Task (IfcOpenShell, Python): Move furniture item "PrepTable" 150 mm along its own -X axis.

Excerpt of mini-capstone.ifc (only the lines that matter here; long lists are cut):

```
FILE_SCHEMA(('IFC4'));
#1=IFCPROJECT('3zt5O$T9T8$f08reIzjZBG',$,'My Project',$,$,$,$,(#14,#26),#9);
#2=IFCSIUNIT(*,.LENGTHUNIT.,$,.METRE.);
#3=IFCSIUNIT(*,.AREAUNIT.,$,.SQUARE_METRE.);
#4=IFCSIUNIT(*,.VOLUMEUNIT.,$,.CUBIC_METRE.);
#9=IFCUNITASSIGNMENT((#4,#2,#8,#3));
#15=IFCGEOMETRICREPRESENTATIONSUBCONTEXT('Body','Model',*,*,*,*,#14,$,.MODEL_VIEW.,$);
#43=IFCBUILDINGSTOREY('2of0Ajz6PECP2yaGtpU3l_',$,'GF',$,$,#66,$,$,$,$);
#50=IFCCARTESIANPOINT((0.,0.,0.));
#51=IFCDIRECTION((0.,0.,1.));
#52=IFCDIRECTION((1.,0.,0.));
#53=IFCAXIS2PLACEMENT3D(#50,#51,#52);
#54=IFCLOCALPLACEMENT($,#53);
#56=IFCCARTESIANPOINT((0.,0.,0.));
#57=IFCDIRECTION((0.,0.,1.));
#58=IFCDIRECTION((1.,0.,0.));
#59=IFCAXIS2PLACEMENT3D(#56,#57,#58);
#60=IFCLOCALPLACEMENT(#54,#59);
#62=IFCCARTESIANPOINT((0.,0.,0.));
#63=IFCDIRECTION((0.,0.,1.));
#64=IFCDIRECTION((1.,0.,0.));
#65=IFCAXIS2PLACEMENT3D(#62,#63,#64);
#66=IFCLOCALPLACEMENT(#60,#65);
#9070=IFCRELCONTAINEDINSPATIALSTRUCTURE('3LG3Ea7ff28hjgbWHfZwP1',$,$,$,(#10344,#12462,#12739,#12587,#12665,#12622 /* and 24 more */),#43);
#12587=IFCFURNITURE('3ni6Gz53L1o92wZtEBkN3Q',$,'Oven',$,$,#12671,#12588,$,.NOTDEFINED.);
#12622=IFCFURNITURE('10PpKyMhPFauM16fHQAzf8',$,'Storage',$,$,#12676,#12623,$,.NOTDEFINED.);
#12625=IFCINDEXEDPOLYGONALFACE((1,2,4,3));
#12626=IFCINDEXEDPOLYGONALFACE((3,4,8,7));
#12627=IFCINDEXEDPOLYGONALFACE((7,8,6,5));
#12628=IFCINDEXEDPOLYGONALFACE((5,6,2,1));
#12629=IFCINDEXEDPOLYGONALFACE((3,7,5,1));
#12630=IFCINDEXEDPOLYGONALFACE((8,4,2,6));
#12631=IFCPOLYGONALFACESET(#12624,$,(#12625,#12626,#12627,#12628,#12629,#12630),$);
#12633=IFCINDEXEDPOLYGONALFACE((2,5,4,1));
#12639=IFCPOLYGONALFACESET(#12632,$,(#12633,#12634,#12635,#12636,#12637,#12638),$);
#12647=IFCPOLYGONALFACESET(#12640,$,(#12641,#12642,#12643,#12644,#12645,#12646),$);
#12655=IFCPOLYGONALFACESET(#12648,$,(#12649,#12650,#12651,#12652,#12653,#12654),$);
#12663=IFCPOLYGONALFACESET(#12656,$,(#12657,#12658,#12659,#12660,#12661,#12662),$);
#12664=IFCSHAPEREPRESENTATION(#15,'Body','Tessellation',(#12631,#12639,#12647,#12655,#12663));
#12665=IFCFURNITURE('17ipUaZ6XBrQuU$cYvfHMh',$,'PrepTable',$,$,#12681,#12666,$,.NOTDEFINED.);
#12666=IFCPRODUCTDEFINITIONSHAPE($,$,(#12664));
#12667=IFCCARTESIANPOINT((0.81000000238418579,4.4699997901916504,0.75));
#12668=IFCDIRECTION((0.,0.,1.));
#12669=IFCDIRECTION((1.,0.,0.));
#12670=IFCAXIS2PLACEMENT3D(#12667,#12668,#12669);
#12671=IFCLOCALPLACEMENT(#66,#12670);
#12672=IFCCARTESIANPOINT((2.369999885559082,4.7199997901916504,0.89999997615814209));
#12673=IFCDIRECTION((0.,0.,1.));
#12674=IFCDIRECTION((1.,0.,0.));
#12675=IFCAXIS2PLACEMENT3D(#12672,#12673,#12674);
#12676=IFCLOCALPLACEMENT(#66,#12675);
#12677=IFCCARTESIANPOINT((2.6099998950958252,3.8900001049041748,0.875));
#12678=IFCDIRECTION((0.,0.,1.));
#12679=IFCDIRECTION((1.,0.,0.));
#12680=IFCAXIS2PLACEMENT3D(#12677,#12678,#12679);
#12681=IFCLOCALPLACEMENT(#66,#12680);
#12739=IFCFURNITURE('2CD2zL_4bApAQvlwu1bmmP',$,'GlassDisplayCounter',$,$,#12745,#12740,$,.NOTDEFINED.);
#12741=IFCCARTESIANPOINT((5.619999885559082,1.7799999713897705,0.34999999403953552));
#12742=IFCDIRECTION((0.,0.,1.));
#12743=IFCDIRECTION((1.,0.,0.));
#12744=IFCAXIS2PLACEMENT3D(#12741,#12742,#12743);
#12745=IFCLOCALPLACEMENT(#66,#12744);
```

```python
import ifcopenshell
import ifcopenshell.api.geometry
import ifcopenshell.util.placement
import ifcopenshell.util.unit

model = ifcopenshell.open("mini-capstone.ifc")
unit_scale = ifcopenshell.util.unit.calculate_unit_scale(model)

item = model.by_guid("17ipUaZ6XBrQuU$cYvfHMh")
matrix = ifcopenshell.util.placement.get_local_placement(item.ObjectPlacement)
matrix[:3, 3] -= matrix[:3, 0] * 0.15 / unit_scale
ifcopenshell.api.geometry.edit_object_placement(model, product=item, matrix=matrix, is_si=False)

print(ifcopenshell.util.placement.get_local_placement(item.ObjectPlacement).round(3) + 0.0)

model.write("mini-capstone_rev.ifc")
```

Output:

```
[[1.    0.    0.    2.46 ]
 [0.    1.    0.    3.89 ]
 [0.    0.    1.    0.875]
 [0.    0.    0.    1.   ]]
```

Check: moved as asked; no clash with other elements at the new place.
